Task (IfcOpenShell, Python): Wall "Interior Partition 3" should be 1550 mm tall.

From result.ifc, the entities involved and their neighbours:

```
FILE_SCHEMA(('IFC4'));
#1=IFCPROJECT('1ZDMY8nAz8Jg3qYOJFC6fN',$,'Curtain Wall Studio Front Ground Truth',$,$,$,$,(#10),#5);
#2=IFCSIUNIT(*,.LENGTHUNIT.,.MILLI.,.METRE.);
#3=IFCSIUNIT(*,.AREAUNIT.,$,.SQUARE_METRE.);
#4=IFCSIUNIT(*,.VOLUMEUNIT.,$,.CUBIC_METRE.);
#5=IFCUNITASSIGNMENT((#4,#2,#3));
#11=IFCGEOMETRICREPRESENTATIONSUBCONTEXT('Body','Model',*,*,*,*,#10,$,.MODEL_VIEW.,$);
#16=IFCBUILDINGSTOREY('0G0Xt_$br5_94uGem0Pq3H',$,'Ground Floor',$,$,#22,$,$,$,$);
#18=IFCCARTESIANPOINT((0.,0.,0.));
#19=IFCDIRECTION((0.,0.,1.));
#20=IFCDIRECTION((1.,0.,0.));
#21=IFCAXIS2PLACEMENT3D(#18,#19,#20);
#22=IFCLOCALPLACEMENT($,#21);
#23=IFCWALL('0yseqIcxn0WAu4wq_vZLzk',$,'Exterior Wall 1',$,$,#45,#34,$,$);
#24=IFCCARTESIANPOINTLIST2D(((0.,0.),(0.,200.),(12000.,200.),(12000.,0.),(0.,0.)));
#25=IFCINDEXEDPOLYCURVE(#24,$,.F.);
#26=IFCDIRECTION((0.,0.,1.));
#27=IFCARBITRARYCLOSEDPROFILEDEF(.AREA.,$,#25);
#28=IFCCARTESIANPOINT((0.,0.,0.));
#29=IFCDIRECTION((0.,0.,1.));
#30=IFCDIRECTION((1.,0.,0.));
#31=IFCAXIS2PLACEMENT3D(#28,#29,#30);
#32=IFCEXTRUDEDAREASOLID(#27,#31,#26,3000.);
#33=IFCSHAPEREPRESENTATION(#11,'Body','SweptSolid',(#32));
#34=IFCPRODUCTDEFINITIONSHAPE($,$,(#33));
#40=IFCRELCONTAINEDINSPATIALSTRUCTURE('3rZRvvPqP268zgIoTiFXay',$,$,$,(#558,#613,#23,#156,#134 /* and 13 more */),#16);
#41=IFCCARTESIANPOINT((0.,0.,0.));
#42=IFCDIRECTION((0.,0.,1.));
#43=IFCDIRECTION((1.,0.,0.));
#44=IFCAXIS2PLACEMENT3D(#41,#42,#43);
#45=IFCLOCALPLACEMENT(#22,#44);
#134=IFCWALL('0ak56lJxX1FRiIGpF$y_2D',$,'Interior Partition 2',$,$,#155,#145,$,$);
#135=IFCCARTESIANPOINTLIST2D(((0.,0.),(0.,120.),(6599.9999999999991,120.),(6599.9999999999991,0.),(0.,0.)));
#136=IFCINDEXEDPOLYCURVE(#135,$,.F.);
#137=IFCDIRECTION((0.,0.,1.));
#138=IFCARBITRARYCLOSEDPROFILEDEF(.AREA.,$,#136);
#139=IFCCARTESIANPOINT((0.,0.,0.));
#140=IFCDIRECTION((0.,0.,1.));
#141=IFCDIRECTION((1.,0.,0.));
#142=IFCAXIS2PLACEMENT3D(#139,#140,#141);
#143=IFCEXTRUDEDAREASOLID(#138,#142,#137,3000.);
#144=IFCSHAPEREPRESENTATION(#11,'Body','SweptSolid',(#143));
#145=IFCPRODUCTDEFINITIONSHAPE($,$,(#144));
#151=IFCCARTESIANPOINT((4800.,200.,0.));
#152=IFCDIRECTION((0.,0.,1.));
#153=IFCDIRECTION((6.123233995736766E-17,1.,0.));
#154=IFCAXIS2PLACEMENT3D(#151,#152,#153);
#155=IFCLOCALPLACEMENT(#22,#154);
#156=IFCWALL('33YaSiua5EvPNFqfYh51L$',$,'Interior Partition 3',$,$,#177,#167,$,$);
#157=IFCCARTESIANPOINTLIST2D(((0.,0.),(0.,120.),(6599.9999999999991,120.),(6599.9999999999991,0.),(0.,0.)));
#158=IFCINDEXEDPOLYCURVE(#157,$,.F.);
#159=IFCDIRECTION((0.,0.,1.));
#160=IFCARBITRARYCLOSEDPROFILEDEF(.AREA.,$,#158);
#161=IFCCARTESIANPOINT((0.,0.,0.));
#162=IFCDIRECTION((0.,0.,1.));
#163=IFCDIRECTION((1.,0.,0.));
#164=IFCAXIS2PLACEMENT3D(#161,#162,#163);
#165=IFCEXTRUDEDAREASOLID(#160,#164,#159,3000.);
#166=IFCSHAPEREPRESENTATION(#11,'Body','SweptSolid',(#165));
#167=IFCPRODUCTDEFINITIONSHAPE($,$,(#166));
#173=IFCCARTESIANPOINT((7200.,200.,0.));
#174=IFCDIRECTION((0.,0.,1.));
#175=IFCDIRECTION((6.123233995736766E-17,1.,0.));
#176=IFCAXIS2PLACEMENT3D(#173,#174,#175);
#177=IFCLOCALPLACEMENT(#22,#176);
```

```python
import ifcopenshell
import ifcopenshell.geom
import ifcopenshell.util.representation
import ifcopenshell.util.shape

model = ifcopenshell.open("result.ifc")
settings = ifcopenshell.geom.settings()


def volume(element):
    """Net volume in cubic metres, openings subtracted."""
    shape = ifcopenshell.geom.create_shape(settings, element)
    return ifcopenshell.util.shape.get_volume(shape.geometry)


wall = model.by_id(156)
before = volume(wall)

body = ifcopenshell.util.representation.get_representation(wall, "Model", "Body")
solid = body.Items[0]
old_height = solid.Depth
solid.Depth = 1550.0
after = volume(wall)

print(f"height {old_height:g} -> {solid.Depth:g}, volume {before:.3f} -> {after:.3f} m3")

model.write("result_v2.ifc")
```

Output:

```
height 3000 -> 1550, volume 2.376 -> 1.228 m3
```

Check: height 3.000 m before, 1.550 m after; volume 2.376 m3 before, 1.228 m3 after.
